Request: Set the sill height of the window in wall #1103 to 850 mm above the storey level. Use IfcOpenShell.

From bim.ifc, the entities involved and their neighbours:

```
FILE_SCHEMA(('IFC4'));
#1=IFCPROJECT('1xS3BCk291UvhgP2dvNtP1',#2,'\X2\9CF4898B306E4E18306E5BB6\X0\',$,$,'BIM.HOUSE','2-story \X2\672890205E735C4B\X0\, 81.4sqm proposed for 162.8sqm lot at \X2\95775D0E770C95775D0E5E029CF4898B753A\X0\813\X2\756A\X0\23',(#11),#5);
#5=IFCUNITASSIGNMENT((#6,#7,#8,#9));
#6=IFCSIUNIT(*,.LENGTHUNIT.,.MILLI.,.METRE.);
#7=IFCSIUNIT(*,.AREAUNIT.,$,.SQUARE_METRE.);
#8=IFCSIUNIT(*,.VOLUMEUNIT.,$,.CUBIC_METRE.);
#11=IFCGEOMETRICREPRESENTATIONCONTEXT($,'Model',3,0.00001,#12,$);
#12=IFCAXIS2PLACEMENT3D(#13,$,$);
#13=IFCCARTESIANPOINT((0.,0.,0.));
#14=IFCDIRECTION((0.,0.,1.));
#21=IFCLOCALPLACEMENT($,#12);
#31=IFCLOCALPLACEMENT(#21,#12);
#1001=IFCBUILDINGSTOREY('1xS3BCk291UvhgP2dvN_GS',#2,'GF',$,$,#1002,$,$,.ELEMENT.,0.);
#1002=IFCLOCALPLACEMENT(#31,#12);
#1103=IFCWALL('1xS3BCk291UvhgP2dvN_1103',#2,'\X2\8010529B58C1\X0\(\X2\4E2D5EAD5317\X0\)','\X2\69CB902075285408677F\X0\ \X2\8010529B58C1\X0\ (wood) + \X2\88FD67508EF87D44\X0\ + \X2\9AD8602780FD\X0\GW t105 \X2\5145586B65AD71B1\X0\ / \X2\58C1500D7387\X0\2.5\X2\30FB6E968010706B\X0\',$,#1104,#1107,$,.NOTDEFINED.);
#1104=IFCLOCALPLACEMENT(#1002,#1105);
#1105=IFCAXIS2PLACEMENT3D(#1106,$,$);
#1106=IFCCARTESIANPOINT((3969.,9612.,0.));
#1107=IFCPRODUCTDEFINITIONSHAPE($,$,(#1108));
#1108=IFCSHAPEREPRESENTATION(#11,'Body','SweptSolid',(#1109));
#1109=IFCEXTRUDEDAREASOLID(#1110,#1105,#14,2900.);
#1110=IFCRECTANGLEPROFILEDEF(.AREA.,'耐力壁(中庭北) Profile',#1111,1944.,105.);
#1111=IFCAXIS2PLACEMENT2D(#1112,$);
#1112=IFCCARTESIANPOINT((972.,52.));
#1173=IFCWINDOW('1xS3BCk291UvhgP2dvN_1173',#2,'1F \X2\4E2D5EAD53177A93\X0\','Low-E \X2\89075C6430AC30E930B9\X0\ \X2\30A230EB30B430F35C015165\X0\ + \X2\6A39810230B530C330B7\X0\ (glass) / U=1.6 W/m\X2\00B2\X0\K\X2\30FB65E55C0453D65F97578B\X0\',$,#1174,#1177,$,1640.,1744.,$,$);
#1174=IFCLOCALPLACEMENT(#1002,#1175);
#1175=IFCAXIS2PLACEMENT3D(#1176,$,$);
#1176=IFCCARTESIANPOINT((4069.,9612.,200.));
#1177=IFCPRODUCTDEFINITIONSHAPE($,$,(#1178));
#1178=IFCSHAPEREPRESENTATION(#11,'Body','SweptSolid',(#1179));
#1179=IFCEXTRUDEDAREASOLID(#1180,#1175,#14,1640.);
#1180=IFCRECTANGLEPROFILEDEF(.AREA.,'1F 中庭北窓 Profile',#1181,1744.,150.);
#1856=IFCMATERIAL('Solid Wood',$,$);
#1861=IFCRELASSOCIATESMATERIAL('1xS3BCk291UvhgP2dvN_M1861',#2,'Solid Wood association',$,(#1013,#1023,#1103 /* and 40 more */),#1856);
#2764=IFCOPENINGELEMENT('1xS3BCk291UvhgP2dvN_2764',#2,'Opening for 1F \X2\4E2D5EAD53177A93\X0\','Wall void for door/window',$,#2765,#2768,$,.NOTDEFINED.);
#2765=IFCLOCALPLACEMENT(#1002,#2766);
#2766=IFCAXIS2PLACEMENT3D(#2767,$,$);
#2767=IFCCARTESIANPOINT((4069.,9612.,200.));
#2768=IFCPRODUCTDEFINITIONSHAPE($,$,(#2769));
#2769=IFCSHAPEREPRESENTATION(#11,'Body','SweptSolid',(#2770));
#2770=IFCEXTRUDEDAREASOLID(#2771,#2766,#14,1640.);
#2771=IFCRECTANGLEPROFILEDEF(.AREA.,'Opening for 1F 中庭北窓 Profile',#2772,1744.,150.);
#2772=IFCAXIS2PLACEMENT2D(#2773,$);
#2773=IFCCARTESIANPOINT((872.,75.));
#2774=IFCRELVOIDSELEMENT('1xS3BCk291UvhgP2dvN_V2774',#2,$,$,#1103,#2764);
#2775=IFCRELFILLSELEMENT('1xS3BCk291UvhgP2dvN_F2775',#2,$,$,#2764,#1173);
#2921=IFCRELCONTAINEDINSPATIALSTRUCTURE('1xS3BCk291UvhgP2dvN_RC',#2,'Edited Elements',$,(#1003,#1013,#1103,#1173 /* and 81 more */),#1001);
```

```python
import numpy as np
import ifcopenshell
import ifcopenshell.api.geometry
import ifcopenshell.geom
import ifcopenshell.util.element
import ifcopenshell.util.placement
import ifcopenshell.util.shape
import ifcopenshell.util.unit

model = ifcopenshell.open("bim.ifc")
unit_scale = ifcopenshell.util.unit.calculate_unit_scale(model)

window = model.by_id(1173)
opening = window.FillsVoids[0].RelatingOpeningElement
storey = ifcopenshell.util.element.get_container(window, ifc_class="IfcBuildingStorey")
level = ifcopenshell.util.placement.get_local_placement(storey.ObjectPlacement)[2, 3]

# The opening's origin need not be at the sill, so measure its lowest point.
shape = ifcopenshell.geom.create_shape(ifcopenshell.geom.settings(), opening)
bottom = ifcopenshell.util.shape.get_shape_bottom_elevation(shape, shape.geometry) / unit_scale
dz = level + 0.85 / unit_scale - bottom

shift = np.array([0.0, 0.0, dz])
# The window is not placed relative to its opening, so move both.
for product in (opening, window):
    matrix = ifcopenshell.util.placement.get_local_placement(product.ObjectPlacement)
    matrix[:3, 3] += shift
    ifcopenshell.api.geometry.edit_object_placement(model, product=product, matrix=matrix, is_si=False)

print(f"moved by {dz * unit_scale:+.3f} m")

model.write("bim_edited.ifc")
```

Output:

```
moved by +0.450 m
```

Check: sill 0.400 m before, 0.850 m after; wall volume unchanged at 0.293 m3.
